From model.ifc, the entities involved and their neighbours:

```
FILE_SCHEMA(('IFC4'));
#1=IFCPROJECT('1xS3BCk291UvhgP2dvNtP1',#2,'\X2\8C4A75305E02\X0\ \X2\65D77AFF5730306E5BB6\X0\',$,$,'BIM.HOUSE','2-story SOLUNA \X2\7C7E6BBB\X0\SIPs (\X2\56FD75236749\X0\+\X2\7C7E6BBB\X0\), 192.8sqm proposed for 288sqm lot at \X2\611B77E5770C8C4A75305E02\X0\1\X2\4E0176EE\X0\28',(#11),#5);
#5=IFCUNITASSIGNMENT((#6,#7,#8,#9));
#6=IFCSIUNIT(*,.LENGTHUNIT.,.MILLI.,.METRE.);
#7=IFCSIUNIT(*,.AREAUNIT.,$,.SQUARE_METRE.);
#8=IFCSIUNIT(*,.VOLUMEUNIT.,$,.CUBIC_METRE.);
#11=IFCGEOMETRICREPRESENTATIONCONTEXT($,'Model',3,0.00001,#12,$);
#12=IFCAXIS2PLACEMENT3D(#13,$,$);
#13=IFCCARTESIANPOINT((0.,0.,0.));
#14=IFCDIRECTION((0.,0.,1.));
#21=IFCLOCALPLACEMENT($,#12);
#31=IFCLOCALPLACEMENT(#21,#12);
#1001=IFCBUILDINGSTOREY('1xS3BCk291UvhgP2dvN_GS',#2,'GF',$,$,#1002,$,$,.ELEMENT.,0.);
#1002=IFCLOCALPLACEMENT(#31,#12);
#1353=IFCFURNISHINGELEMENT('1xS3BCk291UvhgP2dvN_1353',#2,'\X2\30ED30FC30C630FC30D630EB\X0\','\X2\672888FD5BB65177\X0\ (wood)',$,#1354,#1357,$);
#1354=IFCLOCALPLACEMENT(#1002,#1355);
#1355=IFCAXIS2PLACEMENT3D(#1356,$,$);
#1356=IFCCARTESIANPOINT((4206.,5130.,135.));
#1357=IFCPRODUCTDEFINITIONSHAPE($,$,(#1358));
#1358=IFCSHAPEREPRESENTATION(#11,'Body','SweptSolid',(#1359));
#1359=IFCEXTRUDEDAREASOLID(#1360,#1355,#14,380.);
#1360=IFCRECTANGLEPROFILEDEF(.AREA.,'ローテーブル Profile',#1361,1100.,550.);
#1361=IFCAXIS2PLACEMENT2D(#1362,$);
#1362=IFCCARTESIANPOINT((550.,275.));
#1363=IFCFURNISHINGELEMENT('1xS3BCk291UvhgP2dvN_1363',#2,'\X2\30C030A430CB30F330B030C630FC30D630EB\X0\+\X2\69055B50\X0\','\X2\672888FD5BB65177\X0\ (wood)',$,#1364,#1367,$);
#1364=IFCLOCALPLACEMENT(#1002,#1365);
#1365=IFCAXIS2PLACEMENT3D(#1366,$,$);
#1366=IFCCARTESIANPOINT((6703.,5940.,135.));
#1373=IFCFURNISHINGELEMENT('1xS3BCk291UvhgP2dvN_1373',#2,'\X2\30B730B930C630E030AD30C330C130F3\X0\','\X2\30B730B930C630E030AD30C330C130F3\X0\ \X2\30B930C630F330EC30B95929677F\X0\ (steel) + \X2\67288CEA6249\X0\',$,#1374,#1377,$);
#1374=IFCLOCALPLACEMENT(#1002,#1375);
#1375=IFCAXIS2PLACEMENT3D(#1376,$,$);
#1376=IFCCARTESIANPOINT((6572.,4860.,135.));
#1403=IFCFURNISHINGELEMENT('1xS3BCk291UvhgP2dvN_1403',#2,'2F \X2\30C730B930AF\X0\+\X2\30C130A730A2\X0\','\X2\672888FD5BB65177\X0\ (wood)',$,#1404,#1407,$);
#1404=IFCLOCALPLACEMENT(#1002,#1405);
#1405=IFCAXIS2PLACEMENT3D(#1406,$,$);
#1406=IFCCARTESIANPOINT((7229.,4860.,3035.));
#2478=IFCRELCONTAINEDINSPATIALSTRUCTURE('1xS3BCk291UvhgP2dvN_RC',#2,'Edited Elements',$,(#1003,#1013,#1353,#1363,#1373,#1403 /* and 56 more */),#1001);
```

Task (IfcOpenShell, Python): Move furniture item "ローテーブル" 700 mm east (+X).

```python
import ifcopenshell
import ifcopenshell.api.geometry
import ifcopenshell.util.placement
import ifcopenshell.util.unit

model = ifcopenshell.open("model.ifc")
unit_scale = ifcopenshell.util.unit.calculate_unit_scale(model)

item = model.by_guid("1xS3BCk291UvhgP2dvN_1353")
matrix = ifcopenshell.util.placement.get_local_placement(item.ObjectPlacement)
matrix[0, 3] += 0.7 / unit_scale
ifcopenshell.api.geometry.edit_object_placement(model, product=item, matrix=matrix, is_si=False)

print(ifcopenshell.util.placement.get_local_placement(item.ObjectPlacement).round(3) + 0.0)

model.write("model_v2.ifc")
```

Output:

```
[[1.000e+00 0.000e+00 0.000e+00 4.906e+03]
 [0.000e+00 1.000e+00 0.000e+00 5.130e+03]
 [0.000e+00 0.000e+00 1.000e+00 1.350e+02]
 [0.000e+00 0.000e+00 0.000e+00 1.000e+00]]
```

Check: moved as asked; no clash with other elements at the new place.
